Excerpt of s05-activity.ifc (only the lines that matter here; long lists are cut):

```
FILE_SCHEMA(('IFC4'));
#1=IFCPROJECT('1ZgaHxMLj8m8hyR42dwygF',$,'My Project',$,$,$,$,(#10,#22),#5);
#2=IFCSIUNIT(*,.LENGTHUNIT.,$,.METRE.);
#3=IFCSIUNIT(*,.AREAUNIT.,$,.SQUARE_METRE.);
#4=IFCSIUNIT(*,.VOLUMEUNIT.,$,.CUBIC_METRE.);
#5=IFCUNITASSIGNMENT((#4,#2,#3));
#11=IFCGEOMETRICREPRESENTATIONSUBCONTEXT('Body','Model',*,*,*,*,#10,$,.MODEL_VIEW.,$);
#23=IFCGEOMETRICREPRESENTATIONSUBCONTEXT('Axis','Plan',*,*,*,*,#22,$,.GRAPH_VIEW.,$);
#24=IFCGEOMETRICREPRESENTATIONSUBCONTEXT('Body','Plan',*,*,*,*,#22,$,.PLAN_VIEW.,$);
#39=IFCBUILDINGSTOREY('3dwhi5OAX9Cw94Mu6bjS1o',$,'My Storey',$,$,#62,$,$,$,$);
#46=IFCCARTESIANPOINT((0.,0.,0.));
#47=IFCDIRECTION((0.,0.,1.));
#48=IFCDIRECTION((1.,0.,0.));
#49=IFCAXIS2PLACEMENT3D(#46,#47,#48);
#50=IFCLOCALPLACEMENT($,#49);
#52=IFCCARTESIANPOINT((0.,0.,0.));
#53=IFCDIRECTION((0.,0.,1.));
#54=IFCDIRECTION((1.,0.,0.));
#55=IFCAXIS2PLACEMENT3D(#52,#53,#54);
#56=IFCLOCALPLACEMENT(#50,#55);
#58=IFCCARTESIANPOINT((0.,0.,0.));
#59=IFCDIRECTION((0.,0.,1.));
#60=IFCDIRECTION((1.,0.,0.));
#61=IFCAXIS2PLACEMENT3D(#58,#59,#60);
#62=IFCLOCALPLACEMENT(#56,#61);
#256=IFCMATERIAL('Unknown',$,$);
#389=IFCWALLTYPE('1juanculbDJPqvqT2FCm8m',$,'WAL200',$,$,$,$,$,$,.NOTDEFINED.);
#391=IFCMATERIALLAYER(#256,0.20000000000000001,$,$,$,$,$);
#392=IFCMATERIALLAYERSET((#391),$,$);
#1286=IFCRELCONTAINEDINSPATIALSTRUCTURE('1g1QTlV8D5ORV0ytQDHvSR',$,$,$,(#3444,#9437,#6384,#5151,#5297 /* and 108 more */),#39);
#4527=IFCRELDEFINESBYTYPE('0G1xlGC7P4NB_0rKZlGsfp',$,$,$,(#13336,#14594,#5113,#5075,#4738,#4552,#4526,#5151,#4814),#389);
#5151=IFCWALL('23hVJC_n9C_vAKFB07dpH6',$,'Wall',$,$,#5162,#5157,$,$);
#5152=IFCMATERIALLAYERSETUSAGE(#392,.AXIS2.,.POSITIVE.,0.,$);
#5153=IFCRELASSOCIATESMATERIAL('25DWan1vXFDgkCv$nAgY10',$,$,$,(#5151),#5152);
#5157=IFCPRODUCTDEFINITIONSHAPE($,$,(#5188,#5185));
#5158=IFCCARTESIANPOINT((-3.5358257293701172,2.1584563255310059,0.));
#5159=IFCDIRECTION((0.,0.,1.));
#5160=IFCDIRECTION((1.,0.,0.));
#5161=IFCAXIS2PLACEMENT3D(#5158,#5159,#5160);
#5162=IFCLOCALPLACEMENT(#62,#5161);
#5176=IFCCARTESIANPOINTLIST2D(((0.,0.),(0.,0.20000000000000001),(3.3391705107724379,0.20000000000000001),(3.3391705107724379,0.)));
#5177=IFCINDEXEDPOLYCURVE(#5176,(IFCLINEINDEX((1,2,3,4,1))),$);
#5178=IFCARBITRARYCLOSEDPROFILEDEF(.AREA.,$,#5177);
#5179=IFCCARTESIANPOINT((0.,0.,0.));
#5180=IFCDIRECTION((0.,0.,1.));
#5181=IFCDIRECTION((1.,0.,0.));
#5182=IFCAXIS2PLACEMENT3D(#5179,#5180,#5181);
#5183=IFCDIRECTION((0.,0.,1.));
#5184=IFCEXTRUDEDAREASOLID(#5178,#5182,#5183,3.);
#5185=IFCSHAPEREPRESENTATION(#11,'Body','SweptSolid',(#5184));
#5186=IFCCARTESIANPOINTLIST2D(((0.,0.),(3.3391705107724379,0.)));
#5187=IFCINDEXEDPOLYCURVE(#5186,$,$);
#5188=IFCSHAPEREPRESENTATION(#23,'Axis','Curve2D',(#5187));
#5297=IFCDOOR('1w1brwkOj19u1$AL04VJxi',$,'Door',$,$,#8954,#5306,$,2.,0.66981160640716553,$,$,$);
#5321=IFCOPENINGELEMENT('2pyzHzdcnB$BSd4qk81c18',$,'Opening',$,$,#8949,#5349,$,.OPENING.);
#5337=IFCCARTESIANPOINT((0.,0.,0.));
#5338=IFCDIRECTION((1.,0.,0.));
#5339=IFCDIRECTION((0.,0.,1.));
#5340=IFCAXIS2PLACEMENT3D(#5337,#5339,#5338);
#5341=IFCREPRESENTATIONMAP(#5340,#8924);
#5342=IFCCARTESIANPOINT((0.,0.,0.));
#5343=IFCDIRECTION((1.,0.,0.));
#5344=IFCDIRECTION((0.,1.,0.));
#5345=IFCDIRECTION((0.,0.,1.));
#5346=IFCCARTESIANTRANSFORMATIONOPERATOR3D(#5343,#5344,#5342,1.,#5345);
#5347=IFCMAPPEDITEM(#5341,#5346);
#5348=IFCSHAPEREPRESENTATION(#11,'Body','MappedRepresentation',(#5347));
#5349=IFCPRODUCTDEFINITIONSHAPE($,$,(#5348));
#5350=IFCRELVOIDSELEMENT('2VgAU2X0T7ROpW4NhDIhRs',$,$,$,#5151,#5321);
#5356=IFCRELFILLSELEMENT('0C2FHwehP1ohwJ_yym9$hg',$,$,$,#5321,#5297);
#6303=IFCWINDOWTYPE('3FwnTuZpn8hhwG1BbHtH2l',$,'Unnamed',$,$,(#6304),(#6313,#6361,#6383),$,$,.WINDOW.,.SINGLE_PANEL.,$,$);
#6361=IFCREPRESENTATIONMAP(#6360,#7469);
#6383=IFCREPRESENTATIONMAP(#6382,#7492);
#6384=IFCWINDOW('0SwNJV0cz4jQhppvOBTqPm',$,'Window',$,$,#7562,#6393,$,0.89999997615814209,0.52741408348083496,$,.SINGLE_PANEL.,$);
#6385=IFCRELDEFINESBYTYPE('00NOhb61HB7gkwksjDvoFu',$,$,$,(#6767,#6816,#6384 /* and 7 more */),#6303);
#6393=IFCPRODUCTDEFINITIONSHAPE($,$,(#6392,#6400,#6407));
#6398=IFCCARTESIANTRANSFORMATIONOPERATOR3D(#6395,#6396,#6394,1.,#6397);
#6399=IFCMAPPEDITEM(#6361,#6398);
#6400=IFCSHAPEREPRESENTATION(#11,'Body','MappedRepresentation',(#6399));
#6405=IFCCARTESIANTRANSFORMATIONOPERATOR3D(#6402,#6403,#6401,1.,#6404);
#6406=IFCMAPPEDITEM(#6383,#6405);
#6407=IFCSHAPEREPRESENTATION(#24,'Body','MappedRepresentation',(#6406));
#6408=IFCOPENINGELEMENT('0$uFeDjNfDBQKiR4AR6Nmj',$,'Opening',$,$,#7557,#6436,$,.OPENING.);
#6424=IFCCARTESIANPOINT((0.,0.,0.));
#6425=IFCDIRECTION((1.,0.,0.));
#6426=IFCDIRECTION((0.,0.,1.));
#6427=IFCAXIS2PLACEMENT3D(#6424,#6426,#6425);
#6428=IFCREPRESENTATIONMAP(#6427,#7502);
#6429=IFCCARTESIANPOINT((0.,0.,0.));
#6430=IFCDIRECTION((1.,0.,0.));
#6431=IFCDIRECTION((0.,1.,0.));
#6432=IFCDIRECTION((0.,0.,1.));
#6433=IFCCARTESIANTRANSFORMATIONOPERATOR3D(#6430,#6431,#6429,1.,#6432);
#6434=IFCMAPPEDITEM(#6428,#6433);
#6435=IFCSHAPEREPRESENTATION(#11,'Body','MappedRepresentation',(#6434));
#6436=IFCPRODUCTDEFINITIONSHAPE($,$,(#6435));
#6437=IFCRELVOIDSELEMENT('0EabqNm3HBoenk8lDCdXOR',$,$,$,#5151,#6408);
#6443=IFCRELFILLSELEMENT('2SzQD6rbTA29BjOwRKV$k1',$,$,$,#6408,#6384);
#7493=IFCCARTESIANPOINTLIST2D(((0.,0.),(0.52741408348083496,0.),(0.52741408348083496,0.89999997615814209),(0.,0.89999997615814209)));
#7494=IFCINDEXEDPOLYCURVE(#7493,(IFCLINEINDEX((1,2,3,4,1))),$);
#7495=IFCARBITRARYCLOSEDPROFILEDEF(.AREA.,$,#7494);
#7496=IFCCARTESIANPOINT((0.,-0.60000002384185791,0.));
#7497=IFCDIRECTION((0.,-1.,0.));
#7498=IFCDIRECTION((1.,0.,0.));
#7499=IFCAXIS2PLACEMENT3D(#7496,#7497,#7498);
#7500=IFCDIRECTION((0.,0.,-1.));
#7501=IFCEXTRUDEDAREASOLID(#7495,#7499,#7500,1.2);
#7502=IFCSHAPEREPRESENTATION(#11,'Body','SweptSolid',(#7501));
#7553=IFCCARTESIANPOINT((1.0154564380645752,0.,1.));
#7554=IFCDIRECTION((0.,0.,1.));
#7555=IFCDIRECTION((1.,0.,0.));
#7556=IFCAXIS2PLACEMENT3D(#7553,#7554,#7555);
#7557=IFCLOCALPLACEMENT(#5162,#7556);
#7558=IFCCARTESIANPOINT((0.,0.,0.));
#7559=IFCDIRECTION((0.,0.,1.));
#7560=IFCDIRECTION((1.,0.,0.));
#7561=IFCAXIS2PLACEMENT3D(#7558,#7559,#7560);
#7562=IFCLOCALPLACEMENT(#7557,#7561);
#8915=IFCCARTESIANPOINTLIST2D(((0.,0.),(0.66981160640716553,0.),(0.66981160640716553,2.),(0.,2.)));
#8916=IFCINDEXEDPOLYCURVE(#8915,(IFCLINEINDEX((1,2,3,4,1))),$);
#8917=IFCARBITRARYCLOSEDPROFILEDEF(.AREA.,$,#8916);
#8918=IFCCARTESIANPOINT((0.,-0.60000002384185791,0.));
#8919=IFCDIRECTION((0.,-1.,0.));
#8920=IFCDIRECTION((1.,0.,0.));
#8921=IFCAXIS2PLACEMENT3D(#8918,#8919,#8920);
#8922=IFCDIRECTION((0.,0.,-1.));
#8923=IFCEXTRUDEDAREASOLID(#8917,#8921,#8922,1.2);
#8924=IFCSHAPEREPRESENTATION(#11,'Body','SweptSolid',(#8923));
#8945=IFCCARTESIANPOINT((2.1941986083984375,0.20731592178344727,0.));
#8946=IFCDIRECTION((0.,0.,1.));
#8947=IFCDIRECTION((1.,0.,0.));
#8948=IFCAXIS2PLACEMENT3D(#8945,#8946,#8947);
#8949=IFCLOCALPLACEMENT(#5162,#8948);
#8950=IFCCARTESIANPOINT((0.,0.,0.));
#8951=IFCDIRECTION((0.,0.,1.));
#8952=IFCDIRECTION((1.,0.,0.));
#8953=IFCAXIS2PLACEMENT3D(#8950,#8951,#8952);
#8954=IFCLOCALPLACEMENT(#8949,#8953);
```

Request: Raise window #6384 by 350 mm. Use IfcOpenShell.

```python
import numpy as np
import ifcopenshell
import ifcopenshell.api.geometry
import ifcopenshell.util.placement
import ifcopenshell.util.unit

model = ifcopenshell.open("s05-activity.ifc")
unit_scale = ifcopenshell.util.unit.calculate_unit_scale(model)

window = model.by_id(6384)
opening = window.FillsVoids[0].RelatingOpeningElement
dz = 0.35

shift = np.array([0.0, 0.0, dz])
# The window is placed relative to its opening, so it follows when the opening moves.
matrix = ifcopenshell.util.placement.get_local_placement(opening.ObjectPlacement)
matrix[:3, 3] += shift
ifcopenshell.api.geometry.edit_object_placement(
    model, product=opening, matrix=matrix, is_si=False, should_transform_children=True
)

print(f"moved by {dz * unit_scale:+.3f} m")

model.write("s05-activity_edited.ifc")
```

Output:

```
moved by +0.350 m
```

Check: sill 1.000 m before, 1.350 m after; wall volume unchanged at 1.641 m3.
